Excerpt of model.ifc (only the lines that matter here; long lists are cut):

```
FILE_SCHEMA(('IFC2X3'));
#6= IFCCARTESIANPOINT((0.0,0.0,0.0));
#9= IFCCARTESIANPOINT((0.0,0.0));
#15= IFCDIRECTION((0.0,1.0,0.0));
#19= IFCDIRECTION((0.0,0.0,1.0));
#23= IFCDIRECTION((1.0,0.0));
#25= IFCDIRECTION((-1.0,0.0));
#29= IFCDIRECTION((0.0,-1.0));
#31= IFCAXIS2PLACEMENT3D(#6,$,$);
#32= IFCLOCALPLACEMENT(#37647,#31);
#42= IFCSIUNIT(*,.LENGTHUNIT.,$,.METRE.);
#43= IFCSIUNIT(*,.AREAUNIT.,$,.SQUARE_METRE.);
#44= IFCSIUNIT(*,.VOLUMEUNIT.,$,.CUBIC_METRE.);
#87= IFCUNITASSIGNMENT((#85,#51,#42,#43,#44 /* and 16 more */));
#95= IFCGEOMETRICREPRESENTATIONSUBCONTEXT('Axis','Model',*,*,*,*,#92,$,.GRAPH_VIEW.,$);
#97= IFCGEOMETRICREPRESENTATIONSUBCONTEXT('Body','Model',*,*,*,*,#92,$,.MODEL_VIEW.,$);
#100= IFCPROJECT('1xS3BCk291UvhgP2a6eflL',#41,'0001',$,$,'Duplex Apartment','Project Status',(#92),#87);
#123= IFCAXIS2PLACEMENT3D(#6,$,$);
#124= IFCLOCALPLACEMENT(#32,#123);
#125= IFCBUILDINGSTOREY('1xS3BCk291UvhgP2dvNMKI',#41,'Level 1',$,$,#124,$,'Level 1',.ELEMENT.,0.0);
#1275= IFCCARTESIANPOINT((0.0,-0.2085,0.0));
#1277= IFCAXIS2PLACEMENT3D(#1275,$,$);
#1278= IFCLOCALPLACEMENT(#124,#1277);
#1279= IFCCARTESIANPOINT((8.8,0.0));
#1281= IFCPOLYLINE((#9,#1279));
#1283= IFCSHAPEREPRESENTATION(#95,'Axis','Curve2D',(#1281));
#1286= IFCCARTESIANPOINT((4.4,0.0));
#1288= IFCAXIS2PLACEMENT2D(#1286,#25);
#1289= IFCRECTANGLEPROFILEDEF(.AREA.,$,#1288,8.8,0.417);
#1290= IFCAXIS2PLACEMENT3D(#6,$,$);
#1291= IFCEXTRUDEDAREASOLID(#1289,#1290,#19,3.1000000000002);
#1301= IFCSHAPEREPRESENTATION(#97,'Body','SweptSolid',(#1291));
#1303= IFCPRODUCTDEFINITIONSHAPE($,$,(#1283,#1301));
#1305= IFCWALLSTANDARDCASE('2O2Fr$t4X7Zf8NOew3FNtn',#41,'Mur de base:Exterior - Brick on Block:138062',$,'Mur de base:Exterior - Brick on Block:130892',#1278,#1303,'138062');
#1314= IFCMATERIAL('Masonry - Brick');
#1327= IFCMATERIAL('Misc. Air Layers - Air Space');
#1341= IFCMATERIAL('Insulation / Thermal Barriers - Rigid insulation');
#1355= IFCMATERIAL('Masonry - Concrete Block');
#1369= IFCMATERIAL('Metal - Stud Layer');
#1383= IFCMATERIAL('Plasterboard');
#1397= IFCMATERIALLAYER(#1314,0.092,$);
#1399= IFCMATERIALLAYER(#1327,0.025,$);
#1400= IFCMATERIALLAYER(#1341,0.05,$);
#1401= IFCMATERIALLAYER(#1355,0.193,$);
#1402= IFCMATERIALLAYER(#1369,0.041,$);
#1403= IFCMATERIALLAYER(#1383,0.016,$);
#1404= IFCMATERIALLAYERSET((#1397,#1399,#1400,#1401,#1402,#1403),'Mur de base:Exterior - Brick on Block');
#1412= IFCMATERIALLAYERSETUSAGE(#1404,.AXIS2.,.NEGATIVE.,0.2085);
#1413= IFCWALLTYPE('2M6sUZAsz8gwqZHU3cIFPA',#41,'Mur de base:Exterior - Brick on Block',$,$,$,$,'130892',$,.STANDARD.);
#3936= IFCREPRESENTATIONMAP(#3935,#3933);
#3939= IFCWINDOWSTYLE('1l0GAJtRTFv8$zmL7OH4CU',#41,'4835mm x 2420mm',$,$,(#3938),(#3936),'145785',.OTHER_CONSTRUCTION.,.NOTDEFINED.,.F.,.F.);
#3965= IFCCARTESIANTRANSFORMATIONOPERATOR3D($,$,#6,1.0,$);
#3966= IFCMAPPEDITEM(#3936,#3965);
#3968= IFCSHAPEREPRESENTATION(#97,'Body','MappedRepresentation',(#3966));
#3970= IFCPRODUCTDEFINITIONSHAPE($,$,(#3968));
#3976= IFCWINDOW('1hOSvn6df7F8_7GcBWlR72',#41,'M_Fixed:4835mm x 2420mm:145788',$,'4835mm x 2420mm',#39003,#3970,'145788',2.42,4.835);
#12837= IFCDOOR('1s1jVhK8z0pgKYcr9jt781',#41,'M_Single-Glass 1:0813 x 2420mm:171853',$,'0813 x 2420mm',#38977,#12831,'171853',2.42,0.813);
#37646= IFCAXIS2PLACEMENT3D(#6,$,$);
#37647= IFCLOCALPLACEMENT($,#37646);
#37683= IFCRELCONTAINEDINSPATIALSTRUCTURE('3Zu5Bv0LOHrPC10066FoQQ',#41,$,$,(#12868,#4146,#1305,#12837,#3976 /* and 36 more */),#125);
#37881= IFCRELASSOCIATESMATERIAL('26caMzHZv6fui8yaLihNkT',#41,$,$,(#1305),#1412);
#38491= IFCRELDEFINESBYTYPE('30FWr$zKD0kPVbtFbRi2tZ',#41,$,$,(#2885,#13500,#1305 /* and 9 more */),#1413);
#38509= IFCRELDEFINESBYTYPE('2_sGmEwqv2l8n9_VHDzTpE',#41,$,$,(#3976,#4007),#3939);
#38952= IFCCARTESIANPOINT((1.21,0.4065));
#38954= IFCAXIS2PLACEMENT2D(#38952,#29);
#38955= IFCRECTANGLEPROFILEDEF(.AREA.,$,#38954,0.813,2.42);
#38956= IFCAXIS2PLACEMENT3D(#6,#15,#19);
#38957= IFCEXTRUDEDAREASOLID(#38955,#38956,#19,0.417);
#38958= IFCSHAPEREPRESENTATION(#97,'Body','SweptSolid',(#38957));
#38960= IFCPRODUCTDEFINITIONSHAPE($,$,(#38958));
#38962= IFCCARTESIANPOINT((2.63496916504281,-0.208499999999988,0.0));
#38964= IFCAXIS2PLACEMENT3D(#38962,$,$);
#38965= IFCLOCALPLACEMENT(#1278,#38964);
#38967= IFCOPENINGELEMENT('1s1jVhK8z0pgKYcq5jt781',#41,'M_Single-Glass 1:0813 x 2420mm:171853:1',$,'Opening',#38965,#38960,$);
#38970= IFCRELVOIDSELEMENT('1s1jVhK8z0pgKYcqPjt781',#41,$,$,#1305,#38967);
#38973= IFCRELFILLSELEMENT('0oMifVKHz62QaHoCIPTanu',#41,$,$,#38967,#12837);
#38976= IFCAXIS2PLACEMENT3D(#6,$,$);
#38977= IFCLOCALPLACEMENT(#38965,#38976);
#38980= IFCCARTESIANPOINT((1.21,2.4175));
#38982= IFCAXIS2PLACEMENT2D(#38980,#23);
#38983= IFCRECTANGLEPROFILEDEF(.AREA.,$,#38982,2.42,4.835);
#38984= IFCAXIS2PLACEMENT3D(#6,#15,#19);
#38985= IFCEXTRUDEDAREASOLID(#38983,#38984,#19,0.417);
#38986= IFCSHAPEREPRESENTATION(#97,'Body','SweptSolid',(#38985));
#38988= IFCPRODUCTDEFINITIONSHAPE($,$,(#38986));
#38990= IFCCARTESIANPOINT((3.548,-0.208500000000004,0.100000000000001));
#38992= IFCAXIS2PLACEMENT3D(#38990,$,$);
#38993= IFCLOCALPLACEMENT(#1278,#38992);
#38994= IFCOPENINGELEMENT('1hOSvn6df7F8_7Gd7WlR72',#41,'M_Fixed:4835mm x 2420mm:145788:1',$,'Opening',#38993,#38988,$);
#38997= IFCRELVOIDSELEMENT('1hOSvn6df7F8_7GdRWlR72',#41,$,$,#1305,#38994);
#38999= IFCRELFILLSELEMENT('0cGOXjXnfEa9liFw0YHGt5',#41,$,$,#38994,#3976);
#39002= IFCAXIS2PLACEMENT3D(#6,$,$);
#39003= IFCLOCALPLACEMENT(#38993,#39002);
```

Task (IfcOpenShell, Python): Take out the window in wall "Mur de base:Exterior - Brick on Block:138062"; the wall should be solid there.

```python
import ifcopenshell
import ifcopenshell.api.feature
import ifcopenshell.api.root
import ifcopenshell.geom
import ifcopenshell.util.shape

model = ifcopenshell.open("model.ifc")
settings = ifcopenshell.geom.settings()


def volume(element):
    """Net volume in cubic metres, openings subtracted."""
    shape = ifcopenshell.geom.create_shape(settings, element)
    return ifcopenshell.util.shape.get_volume(shape.geometry)


window = model.by_guid("1hOSvn6df7F8_7GcBWlR72")
opening = window.FillsVoids[0].RelatingOpeningElement
wall = opening.VoidsElements[0].RelatingBuildingElement
before = volume(wall)

ifcopenshell.api.root.remove_product(model, product=window)
ifcopenshell.api.feature.remove_feature(model, feature=opening)

after = volume(wall)

print(f"wall volume {before:.3f} -> {after:.3f} m3")

model.write("model_updated.ifc")
```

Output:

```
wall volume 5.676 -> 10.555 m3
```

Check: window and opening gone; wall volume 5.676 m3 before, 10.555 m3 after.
